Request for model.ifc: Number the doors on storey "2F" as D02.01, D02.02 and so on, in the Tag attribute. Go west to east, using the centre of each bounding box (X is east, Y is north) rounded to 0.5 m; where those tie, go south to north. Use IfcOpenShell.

First a look at what the model holds.

```python
import ifcopenshell
import ifcopenshell.util.element
import ifcopenshell.util.placement

model = ifcopenshell.open("model.ifc")
print(model.schema)
storey = next(s for s in model.by_type("IfcBuildingStorey") if s.Name == "2F")
doors = [e for e in ifcopenshell.util.element.get_decomposition(storey) if e.is_a("IfcDoor")]
for e in sorted(doors, key=lambda e: e.id()):
    origin = ifcopenshell.util.placement.get_local_placement(e.ObjectPlacement)[:3, 3]
    print(e.id(), e.Tag, e.Name, origin.round(2) + 0.0, sep=" | ")
```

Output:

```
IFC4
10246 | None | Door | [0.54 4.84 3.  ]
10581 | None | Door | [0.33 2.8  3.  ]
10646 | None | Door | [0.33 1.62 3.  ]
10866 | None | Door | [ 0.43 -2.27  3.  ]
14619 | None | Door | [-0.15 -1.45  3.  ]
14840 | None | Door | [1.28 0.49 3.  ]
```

```python
import ifcopenshell
import ifcopenshell.geom
import ifcopenshell.util.element
import ifcopenshell.util.shape

model = ifcopenshell.open("model.ifc")
settings = ifcopenshell.geom.settings()
settings.set("use-world-coords", True)


def centre(element):
    shape = ifcopenshell.geom.create_shape(settings, element)
    return ifcopenshell.util.shape.get_bbox_centroid(shape.geometry)


storey = next(s for s in model.by_type("IfcBuildingStorey") if s.Name == "2F")
doors = [e for e in ifcopenshell.util.element.get_decomposition(storey) if e.is_a("IfcDoor")]

# Insertion points can sit at a corner or the storey origin, so sort by the geometry (in metres).
centres = {e: centre(e) for e in doors}
doors.sort(key=lambda e: (round(centres[e][0] / 0.5), centres[e][1]))

for i, e in enumerate(doors, start=1):
    number = f"D02.{i:02d}"
    e.Tag = number
    print(e.id(), number)

model.write("model_rev.ifc")
```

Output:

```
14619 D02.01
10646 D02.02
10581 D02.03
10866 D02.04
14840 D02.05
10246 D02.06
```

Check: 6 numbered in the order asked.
